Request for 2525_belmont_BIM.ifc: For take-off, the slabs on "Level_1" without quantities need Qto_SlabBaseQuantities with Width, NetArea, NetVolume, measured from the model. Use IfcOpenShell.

First a look at what the model holds.

```python
import ifcopenshell
import ifcopenshell.util.element
import ifcopenshell.util.unit

model = ifcopenshell.open("2525_belmont_BIM.ifc")
print(model.schema)
for unit_type in ("LENGTHUNIT", "AREAUNIT", "VOLUMEUNIT"):
    print(unit_type, ifcopenshell.util.unit.calculate_unit_scale(model, unit_type))
storey = next(s for s in model.by_type("IfcBuildingStorey") if s.Name == "Level_1")
slabs = [e for e in ifcopenshell.util.element.get_decomposition(storey) if e.is_a("IfcSlab")]
for e in sorted(slabs, key=lambda e: e.id()):
    print(e.id(), e.is_a(), e.Name, list(ifcopenshell.util.element.get_psets(e, qtos_only=True)), sep=" | ")
```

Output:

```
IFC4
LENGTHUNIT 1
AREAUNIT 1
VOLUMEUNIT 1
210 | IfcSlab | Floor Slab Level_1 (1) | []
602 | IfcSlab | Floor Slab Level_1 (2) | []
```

```python
import ifcopenshell
import ifcopenshell.api.pset
import ifcopenshell.geom
import ifcopenshell.util.element
import ifcopenshell.util.shape
import ifcopenshell.util.unit

model = ifcopenshell.open("2525_belmont_BIM.ifc")
unit_scale = ifcopenshell.util.unit.calculate_unit_scale(model)
area_scale = ifcopenshell.util.unit.calculate_unit_scale(model, "AREAUNIT")
volume_scale = ifcopenshell.util.unit.calculate_unit_scale(model, "VOLUMEUNIT")
settings = ifcopenshell.geom.settings()

storey = next(s for s in model.by_type("IfcBuildingStorey") if s.Name == "Level_1")
slabs = [e for e in ifcopenshell.util.element.get_decomposition(storey) if e.is_a("IfcSlab")]

for e in sorted(slabs, key=lambda e: e.id()):
    if ifcopenshell.util.element.get_psets(e, qtos_only=True, should_inherit=False):
        continue
    # Geometry comes back in metres, in the element's own axes.
    shape = ifcopenshell.geom.create_shape(settings, e)
    values = {
        "Width": ifcopenshell.util.shape.get_z(shape.geometry) / unit_scale,
        "NetArea": ifcopenshell.util.shape.get_footprint_area(shape.geometry) / area_scale,
        "NetVolume": ifcopenshell.util.shape.get_volume(shape.geometry) / volume_scale,
    }
    qto = ifcopenshell.api.pset.add_qto(model, product=e, name="Qto_SlabBaseQuantities")
    ifcopenshell.api.pset.edit_qto(model, qto=qto, properties=values)
    print(e.id(), {k: round(v, 3) for k, v in values.items()})

model.write("2525_belmont_BIM_updated.ifc")
```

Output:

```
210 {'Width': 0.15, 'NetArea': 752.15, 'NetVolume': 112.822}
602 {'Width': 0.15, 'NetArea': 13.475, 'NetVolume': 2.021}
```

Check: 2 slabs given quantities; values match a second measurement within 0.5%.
